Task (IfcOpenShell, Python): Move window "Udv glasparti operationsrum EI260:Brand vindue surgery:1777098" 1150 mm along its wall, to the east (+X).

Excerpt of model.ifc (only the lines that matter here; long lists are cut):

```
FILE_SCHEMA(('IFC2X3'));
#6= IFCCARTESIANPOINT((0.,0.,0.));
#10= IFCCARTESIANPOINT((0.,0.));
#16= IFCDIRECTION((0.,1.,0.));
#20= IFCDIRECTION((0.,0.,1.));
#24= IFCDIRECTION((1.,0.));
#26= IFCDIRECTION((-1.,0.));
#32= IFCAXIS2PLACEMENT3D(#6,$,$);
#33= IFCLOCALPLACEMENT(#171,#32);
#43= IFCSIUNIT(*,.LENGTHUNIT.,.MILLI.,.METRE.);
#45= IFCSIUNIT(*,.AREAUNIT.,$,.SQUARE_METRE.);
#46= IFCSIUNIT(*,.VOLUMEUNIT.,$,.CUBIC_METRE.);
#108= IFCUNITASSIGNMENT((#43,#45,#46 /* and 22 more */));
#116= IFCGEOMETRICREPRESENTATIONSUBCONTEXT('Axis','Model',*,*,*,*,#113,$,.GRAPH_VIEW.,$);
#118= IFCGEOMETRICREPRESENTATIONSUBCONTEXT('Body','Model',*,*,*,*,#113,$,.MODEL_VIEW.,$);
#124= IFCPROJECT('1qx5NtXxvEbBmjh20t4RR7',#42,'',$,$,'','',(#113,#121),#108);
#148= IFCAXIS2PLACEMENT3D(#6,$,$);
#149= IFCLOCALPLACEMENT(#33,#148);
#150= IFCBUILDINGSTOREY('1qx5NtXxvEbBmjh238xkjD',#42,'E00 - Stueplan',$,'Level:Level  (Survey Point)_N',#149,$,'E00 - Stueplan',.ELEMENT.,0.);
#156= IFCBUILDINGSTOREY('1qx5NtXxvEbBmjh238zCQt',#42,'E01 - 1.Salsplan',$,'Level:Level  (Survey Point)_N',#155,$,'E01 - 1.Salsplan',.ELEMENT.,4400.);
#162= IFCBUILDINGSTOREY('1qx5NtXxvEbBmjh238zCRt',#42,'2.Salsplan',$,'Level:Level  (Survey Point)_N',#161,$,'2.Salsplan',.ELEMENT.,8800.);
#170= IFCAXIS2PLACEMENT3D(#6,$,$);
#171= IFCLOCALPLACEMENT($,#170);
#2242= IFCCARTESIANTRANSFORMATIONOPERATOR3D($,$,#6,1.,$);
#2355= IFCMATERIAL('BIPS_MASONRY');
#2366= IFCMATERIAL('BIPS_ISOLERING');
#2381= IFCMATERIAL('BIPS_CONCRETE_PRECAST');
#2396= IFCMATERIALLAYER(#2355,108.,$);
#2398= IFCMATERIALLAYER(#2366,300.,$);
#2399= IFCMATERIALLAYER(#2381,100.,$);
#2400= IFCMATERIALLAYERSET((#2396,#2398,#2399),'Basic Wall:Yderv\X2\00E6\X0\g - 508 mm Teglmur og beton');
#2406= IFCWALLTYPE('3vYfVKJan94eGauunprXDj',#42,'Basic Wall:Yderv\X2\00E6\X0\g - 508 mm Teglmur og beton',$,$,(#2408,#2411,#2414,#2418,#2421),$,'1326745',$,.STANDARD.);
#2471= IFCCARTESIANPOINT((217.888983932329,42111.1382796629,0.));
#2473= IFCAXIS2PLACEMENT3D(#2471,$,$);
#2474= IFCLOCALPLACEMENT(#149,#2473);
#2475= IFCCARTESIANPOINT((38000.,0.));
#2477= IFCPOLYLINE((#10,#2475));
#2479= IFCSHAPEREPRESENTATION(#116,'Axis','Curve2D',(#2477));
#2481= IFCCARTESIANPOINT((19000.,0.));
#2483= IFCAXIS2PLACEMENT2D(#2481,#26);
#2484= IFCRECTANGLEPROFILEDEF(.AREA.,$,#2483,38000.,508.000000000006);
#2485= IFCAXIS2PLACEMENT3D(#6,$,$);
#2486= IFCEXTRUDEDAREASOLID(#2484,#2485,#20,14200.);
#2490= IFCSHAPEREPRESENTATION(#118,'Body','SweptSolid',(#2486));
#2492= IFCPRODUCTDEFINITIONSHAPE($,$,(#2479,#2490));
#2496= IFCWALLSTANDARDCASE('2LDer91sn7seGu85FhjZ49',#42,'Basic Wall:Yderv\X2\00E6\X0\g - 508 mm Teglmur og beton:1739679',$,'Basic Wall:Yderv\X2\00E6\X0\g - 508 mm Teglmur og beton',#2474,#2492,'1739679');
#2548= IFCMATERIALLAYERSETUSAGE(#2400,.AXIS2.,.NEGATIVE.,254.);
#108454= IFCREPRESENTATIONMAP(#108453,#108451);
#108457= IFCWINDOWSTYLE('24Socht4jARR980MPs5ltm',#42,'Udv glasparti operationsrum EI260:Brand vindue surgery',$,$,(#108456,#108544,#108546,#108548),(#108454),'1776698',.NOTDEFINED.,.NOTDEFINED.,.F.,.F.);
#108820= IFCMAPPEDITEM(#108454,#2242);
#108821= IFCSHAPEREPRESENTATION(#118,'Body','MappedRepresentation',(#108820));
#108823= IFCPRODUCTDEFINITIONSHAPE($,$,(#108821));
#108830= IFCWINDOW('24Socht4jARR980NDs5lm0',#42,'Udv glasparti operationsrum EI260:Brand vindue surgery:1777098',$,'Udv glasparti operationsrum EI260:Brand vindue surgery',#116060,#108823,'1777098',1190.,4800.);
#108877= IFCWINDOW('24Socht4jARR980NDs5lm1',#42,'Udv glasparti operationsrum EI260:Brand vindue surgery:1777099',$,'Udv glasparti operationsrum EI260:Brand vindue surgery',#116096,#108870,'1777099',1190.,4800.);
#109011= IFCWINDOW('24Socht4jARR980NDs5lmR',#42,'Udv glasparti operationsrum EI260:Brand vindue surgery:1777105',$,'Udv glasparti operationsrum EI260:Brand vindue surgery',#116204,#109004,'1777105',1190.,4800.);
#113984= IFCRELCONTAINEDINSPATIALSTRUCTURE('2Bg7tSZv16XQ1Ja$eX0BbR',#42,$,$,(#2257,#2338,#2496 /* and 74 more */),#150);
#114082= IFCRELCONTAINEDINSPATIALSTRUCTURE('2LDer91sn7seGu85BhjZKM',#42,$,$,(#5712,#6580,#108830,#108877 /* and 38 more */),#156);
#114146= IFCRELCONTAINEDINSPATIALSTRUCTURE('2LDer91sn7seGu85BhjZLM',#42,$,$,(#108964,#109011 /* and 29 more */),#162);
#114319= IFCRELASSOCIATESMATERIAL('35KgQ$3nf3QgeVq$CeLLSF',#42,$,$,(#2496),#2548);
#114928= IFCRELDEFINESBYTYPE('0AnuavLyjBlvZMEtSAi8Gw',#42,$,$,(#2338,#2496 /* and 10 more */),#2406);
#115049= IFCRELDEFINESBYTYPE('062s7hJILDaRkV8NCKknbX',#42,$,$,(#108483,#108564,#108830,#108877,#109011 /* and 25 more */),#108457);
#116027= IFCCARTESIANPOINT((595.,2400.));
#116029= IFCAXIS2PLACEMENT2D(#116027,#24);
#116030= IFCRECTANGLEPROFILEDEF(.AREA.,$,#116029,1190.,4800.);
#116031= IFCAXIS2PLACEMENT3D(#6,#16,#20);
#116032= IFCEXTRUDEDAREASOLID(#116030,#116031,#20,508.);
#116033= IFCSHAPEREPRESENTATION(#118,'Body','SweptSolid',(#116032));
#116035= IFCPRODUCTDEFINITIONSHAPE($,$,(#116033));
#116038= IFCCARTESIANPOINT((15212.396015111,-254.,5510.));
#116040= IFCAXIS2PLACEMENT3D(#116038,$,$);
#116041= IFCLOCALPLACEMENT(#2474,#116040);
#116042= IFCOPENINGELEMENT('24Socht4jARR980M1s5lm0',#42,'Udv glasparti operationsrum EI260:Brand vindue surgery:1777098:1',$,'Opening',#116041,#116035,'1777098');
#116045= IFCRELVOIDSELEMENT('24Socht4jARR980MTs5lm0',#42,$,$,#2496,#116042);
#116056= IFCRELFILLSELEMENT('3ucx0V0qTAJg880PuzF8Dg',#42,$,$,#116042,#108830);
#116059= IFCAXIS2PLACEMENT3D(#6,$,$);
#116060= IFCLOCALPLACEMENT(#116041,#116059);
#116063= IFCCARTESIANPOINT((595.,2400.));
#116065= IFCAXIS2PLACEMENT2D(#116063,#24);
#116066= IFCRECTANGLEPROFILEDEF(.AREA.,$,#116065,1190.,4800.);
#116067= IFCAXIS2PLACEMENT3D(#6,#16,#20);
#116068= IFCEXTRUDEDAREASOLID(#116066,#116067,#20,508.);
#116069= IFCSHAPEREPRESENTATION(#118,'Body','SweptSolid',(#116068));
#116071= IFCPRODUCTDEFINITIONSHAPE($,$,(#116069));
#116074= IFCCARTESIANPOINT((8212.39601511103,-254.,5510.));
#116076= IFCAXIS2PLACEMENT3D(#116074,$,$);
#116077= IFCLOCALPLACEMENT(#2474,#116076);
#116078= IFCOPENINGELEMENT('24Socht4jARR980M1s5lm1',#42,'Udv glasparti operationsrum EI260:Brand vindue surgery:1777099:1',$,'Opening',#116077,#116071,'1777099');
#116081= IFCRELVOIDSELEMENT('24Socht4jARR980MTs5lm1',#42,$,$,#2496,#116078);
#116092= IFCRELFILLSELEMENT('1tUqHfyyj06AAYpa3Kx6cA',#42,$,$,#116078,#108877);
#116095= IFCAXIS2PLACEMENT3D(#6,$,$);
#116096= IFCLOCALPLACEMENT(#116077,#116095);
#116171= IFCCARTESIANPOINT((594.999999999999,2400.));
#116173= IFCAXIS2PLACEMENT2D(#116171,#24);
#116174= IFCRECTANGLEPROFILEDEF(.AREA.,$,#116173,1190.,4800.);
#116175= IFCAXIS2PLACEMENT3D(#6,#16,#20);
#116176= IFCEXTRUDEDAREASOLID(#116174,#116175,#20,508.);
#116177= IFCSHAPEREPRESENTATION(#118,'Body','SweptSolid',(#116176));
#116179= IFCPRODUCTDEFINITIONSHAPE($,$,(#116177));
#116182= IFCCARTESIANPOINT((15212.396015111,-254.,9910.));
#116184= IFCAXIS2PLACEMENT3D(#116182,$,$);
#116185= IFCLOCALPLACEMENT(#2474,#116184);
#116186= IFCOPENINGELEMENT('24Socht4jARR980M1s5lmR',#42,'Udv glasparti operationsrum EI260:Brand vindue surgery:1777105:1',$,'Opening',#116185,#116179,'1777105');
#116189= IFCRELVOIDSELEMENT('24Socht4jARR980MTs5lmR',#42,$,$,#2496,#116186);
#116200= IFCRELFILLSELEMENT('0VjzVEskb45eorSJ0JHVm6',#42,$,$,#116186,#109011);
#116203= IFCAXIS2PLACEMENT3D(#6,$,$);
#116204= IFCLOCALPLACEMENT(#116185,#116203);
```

```python
import ifcopenshell
import ifcopenshell.api.geometry
import ifcopenshell.util.placement

model = ifcopenshell.open("model.ifc")

window = model.by_guid("24Socht4jARR980NDs5lm0")
opening = window.FillsVoids[0].RelatingOpeningElement
wall = opening.VoidsElements[0].RelatingBuildingElement

wall_matrix = ifcopenshell.util.placement.get_local_placement(wall.ObjectPlacement)
shift = wall_matrix[:3, 0] * 1150.0
before = ifcopenshell.util.placement.get_local_placement(window.ObjectPlacement)[:3, 3].copy()

# The window is placed relative to its opening, so it follows when the opening moves.
matrix = ifcopenshell.util.placement.get_local_placement(opening.ObjectPlacement)
matrix[:3, 3] += shift
ifcopenshell.api.geometry.edit_object_placement(
    model, product=opening, matrix=matrix, is_si=False, should_transform_children=True
)

after = ifcopenshell.util.placement.get_local_placement(window.ObjectPlacement)[:3, 3]
print("window moved by", (after - before).round(3) + 0.0)

model.write("model-out.ifc")
```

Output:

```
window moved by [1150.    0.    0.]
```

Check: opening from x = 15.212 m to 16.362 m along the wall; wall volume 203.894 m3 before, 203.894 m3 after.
